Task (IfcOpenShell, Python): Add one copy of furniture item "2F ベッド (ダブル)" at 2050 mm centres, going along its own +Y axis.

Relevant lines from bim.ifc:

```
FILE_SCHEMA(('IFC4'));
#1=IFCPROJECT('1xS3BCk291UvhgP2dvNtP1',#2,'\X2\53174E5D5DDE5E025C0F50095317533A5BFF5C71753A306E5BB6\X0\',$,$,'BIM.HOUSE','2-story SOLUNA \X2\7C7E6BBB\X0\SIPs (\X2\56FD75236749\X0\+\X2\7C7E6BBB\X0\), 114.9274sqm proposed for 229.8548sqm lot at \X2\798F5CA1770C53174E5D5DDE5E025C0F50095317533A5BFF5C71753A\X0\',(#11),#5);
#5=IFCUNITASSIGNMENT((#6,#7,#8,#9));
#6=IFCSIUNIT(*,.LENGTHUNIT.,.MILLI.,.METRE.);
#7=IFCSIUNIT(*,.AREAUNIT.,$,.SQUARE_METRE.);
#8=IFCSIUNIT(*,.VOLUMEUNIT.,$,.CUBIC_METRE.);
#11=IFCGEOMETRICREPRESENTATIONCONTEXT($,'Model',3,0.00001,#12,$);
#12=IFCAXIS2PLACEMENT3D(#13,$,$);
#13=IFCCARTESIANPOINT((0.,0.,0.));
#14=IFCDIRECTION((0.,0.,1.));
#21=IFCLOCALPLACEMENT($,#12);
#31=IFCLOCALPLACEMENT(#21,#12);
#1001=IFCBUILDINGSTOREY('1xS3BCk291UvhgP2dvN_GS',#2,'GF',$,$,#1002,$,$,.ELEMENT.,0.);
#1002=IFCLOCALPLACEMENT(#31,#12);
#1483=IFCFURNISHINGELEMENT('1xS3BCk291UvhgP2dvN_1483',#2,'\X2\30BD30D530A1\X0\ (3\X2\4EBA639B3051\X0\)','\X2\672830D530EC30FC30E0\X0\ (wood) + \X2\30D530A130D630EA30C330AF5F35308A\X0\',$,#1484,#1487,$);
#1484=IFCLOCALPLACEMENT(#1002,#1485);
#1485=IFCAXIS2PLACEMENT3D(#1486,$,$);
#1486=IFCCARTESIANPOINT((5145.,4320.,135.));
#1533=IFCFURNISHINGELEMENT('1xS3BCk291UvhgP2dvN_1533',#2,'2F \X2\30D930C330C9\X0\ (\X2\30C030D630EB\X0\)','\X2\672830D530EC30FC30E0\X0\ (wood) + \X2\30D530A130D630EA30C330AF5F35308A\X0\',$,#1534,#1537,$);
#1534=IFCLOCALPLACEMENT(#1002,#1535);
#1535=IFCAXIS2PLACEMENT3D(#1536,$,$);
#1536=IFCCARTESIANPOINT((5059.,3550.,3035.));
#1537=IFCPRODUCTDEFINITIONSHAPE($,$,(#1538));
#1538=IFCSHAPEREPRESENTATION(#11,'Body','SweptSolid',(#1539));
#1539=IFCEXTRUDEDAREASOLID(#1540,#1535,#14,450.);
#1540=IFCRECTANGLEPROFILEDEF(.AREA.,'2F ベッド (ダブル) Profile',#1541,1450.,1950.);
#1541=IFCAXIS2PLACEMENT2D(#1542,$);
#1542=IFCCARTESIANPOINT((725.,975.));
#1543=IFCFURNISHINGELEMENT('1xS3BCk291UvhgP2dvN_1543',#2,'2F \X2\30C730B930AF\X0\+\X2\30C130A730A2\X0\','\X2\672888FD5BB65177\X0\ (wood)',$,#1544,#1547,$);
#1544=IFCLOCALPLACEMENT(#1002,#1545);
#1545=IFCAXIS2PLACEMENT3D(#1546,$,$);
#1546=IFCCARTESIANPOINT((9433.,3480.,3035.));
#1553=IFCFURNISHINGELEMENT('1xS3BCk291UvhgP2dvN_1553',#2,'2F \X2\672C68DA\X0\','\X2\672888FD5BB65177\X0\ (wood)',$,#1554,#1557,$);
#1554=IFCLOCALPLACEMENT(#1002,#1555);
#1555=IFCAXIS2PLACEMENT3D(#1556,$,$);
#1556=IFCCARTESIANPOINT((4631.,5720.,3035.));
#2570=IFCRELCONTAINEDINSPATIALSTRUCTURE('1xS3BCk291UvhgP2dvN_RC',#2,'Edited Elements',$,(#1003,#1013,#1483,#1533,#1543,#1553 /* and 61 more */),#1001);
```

```python
import ifcopenshell
import ifcopenshell.api.geometry
import ifcopenshell.api.root
import ifcopenshell.util.element
import ifcopenshell.util.placement

model = ifcopenshell.open("bim.ifc")


def reuse_history(source, copy):
    """copy_class also copies each property set's owner history, people and application; keep the originals."""
    for rel in copy.IsDefinedBy:
        if rel.is_a("IfcRelDefinesByProperties") and (history := rel.RelatingPropertyDefinition.OwnerHistory):
            rel.RelatingPropertyDefinition.OwnerHistory = source.OwnerHistory
            ifcopenshell.util.element.remove_deep2(model, history)


source = model.by_guid("1xS3BCk291UvhgP2dvN_1533")
base = ifcopenshell.util.placement.get_local_placement(source.ObjectPlacement)
step = base[:3, 1] * 2050.0

for i in range(1, 2):
    copy = ifcopenshell.api.root.copy_class(model, product=source)
    copy.Representation = ifcopenshell.util.element.copy_deep(
        model, source.Representation, exclude=["IfcGeometricRepresentationContext", "IfcRepresentationMap"]
    )
    reuse_history(source, copy)
    matrix = base.copy()
    matrix[:3, 3] += i * step
    print("added at", matrix[:3, 3].round(3) + 0.0)
    ifcopenshell.api.geometry.edit_object_placement(model, product=copy, matrix=matrix, is_si=False)

model.write("bim-out.ifc")
```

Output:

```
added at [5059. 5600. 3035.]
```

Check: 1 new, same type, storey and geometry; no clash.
